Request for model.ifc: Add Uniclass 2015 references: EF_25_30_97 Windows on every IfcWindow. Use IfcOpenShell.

First a look at what the model holds.

```python
import ifcopenshell

model = ifcopenshell.open("model.ifc")
print(model.schema)
print("classifications:", [c.Name for c in model.by_type("IfcClassification")])
for ifc_class in ("IfcDoor", "IfcRoof", "IfcStair", "IfcWall", "IfcWindow"):
    print(ifc_class, len(model.by_type(ifc_class)))
```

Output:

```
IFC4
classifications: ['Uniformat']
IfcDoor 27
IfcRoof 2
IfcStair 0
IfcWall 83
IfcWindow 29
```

```python
import ifcopenshell
import ifcopenshell.api.classification

model = ifcopenshell.open("model.ifc")

system = ifcopenshell.api.classification.add_classification(model, classification="Uniclass 2015")

codes = {
    "IfcWindow": ("EF_25_30_97", "Windows"),
}
for ifc_class, (code, name) in codes.items():
    products = model.by_type(ifc_class)
    ifcopenshell.api.classification.add_reference(
        model, products=products, classification=system, identification=code, name=name
    )
    print(code, len(products))

model.write("model_v2.ifc")
```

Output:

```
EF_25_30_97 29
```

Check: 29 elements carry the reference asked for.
